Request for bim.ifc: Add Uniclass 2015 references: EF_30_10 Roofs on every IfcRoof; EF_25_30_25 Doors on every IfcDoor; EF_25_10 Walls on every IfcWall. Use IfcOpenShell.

First a look at what the model holds.

```python
import ifcopenshell

model = ifcopenshell.open("bim.ifc")
print(model.schema)
print("classifications:", [c.Name for c in model.by_type("IfcClassification")])
for ifc_class in ("IfcDoor", "IfcRoof", "IfcStair", "IfcWall", "IfcWindow"):
    print(ifc_class, len(model.by_type(ifc_class)))
```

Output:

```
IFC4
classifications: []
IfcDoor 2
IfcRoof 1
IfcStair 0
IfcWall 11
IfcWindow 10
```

```python
import ifcopenshell
import ifcopenshell.api.classification

model = ifcopenshell.open("bim.ifc")

system = ifcopenshell.api.classification.add_classification(model, classification="Uniclass 2015")

codes = {
    "IfcRoof": ("EF_30_10", "Roofs"),
    "IfcDoor": ("EF_25_30_25", "Doors"),
    "IfcWall": ("EF_25_10", "Walls"),
}
for ifc_class, (code, name) in codes.items():
    products = model.by_type(ifc_class)
    ifcopenshell.api.classification.add_reference(
        model, products=products, classification=system, identification=code, name=name
    )
    print(code, len(products))

model.write("bim_rev.ifc")
```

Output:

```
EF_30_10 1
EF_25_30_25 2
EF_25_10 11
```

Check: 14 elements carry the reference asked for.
